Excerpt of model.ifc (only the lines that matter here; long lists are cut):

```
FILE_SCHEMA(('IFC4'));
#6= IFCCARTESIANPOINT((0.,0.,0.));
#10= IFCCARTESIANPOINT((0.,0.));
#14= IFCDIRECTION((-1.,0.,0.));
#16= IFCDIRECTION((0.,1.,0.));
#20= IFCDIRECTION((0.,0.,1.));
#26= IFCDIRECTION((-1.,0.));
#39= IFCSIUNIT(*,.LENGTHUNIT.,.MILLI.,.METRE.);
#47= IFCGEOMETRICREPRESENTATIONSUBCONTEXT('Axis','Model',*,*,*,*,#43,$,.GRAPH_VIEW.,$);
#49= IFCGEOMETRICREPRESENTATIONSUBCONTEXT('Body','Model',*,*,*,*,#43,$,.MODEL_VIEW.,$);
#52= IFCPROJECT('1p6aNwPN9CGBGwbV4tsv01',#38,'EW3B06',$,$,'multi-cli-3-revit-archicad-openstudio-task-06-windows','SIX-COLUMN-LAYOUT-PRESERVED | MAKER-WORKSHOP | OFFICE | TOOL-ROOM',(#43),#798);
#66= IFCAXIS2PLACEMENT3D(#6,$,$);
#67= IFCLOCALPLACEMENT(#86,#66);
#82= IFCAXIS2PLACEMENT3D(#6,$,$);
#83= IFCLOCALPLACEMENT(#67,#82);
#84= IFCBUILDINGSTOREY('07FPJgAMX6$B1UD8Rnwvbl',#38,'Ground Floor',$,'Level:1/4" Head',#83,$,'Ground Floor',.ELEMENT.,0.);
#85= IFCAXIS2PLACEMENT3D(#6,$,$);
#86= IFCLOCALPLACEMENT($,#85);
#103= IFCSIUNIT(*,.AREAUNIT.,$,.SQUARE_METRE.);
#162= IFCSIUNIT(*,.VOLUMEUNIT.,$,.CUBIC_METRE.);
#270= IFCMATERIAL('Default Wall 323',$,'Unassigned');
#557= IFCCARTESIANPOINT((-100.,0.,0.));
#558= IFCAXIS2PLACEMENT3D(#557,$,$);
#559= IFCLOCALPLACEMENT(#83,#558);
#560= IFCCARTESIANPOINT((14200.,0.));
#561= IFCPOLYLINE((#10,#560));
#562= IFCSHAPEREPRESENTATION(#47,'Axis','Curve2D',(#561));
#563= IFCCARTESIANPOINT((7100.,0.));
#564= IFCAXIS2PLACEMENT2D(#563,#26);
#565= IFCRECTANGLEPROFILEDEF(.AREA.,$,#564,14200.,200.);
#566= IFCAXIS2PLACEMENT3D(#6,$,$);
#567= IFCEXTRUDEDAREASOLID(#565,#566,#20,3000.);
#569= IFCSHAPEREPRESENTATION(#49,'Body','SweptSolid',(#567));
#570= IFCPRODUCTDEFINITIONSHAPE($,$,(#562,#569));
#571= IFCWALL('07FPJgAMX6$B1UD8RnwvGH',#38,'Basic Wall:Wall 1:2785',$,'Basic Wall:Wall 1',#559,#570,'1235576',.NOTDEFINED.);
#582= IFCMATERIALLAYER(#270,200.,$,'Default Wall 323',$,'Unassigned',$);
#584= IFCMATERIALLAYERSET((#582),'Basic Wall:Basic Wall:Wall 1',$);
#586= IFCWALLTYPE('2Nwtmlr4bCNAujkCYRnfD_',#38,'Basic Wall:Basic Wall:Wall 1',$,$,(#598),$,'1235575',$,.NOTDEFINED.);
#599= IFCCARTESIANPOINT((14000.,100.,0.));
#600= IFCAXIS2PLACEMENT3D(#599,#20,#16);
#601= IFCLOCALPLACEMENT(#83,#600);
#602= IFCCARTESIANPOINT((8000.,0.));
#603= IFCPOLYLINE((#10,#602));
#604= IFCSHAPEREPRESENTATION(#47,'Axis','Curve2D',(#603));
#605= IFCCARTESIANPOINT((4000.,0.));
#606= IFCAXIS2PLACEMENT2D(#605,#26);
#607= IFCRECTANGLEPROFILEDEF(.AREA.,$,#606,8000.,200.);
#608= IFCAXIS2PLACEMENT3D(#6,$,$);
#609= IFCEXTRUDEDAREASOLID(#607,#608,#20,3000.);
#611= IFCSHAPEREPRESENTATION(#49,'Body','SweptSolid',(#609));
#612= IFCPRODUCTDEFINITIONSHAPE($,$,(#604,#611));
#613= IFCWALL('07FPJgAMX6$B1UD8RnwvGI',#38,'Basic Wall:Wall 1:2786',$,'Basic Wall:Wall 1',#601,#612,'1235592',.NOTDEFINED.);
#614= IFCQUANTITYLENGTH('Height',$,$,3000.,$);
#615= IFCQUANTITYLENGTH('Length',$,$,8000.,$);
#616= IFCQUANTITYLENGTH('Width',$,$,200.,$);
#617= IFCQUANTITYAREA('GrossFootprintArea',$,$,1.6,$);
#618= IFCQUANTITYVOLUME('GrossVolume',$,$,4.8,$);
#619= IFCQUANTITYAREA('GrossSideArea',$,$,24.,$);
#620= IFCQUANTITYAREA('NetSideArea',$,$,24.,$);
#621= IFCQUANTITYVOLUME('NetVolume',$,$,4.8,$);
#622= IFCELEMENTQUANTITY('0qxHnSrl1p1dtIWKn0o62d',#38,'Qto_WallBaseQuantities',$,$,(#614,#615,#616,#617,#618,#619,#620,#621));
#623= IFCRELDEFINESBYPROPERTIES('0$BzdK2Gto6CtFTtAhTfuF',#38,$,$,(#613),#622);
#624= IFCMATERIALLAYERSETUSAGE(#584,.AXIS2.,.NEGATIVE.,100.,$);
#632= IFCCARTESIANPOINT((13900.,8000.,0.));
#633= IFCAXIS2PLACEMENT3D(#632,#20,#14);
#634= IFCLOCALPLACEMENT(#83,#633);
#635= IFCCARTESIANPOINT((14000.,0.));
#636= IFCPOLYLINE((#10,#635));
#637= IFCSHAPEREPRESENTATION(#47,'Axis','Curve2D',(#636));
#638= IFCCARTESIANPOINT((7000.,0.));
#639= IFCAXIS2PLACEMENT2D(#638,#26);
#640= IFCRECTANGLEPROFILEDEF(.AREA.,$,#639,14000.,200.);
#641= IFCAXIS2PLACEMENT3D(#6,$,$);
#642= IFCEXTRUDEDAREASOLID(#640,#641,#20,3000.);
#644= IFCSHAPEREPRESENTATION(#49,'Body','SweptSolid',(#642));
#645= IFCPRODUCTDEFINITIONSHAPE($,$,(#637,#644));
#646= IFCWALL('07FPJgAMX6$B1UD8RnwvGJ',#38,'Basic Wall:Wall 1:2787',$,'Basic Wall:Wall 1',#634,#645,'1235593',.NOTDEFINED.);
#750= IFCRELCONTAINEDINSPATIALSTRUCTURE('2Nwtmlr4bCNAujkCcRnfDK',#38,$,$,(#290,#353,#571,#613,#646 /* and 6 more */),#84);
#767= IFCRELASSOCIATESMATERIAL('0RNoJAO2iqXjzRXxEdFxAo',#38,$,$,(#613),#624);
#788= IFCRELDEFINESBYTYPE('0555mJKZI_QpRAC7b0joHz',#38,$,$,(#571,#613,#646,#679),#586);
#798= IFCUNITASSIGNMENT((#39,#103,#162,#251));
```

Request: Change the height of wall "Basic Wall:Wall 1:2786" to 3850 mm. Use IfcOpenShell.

```python
import ifcopenshell
import ifcopenshell.api.pset
import ifcopenshell.geom
import ifcopenshell.util.element
import ifcopenshell.util.representation
import ifcopenshell.util.shape
import ifcopenshell.util.unit

model = ifcopenshell.open("model.ifc")
unit_scale = ifcopenshell.util.unit.calculate_unit_scale(model)
area_scale = ifcopenshell.util.unit.calculate_unit_scale(model, "AREAUNIT")
volume_scale = ifcopenshell.util.unit.calculate_unit_scale(model, "VOLUMEUNIT")
settings = ifcopenshell.geom.settings()


def volume(element):
    """Net volume in cubic metres, openings subtracted."""
    shape = ifcopenshell.geom.create_shape(settings, element)
    return ifcopenshell.util.shape.get_volume(shape.geometry)


wall = model.by_guid("07FPJgAMX6$B1UD8RnwvGI")
before = volume(wall)

body = ifcopenshell.util.representation.get_representation(wall, "Model", "Body")
solid = body.Items[0]
old_height = solid.Depth
solid.Depth = 3.85 / unit_scale
after = volume(wall)
thickness = 0.2  # wall thickness in metres

# Update the stored height, areas and volumes.
qto = model.by_id(ifcopenshell.util.element.get_pset(wall, "Qto_WallBaseQuantities", should_inherit=False)["id"])
ifcopenshell.api.pset.edit_qto(model, qto=qto, properties={
    "Height": solid.Depth,
    "GrossVolume": ifcopenshell.util.element.get_pset(wall, "Qto_WallBaseQuantities", "GrossVolume") * solid.Depth / old_height,
    "GrossSideArea": ifcopenshell.util.element.get_pset(wall, "Qto_WallBaseQuantities", "GrossSideArea") * solid.Depth / old_height,
    "NetSideArea": after / thickness / area_scale,
    "NetVolume": after / volume_scale,
})

print(f"height {old_height:g} -> {solid.Depth:g}, volume {before:.3f} -> {after:.3f} m3")

model.write("model_updated.ifc")
```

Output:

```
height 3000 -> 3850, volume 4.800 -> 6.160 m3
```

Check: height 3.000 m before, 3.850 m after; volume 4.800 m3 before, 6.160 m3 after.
